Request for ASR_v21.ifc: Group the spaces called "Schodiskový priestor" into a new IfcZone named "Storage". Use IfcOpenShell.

First a look at what the model holds.

```python
import ifcopenshell

model = ifcopenshell.open("ASR_v21.ifc")
print(model.schema)
seen = {}
for space in model.by_type("IfcSpace"):
    seen[space.LongName] = seen.get(space.LongName, 0) + 1
for name, count in sorted(seen.items(), key=str):
    print(count, "x", name)
print("zones:", [z.Name for z in model.by_type("IfcZone")][:20])
```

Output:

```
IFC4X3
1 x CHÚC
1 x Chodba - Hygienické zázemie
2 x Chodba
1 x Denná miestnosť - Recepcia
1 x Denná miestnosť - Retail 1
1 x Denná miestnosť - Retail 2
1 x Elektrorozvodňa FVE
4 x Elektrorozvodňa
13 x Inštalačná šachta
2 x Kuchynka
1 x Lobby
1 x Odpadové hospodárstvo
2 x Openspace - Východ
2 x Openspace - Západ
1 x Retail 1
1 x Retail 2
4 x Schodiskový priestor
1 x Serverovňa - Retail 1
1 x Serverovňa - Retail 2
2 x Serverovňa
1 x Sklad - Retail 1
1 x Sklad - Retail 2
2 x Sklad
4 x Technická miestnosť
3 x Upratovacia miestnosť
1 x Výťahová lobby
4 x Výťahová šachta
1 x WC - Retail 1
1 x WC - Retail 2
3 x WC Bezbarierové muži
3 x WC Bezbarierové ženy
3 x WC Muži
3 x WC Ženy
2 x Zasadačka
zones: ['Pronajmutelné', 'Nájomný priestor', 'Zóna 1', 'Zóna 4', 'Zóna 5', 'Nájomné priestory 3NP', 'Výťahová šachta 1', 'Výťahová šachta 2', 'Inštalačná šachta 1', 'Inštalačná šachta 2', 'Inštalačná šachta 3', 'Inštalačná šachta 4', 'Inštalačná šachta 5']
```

```python
import ifcopenshell
import ifcopenshell.api.group
import ifcopenshell.api.root

model = ifcopenshell.open("ASR_v21.ifc")

names = {"Schodiskový priestor"}
spaces = [s for s in model.by_type("IfcSpace") if s.LongName in names]

zone = ifcopenshell.api.root.create_entity(model, ifc_class="IfcZone", name="Storage")
ifcopenshell.api.group.assign_group(model, products=spaces, group=zone)
print(len(spaces), "spaces in", zone.Name)

model.write("ASR_v21_updated.ifc")
```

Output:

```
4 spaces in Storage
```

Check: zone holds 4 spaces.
